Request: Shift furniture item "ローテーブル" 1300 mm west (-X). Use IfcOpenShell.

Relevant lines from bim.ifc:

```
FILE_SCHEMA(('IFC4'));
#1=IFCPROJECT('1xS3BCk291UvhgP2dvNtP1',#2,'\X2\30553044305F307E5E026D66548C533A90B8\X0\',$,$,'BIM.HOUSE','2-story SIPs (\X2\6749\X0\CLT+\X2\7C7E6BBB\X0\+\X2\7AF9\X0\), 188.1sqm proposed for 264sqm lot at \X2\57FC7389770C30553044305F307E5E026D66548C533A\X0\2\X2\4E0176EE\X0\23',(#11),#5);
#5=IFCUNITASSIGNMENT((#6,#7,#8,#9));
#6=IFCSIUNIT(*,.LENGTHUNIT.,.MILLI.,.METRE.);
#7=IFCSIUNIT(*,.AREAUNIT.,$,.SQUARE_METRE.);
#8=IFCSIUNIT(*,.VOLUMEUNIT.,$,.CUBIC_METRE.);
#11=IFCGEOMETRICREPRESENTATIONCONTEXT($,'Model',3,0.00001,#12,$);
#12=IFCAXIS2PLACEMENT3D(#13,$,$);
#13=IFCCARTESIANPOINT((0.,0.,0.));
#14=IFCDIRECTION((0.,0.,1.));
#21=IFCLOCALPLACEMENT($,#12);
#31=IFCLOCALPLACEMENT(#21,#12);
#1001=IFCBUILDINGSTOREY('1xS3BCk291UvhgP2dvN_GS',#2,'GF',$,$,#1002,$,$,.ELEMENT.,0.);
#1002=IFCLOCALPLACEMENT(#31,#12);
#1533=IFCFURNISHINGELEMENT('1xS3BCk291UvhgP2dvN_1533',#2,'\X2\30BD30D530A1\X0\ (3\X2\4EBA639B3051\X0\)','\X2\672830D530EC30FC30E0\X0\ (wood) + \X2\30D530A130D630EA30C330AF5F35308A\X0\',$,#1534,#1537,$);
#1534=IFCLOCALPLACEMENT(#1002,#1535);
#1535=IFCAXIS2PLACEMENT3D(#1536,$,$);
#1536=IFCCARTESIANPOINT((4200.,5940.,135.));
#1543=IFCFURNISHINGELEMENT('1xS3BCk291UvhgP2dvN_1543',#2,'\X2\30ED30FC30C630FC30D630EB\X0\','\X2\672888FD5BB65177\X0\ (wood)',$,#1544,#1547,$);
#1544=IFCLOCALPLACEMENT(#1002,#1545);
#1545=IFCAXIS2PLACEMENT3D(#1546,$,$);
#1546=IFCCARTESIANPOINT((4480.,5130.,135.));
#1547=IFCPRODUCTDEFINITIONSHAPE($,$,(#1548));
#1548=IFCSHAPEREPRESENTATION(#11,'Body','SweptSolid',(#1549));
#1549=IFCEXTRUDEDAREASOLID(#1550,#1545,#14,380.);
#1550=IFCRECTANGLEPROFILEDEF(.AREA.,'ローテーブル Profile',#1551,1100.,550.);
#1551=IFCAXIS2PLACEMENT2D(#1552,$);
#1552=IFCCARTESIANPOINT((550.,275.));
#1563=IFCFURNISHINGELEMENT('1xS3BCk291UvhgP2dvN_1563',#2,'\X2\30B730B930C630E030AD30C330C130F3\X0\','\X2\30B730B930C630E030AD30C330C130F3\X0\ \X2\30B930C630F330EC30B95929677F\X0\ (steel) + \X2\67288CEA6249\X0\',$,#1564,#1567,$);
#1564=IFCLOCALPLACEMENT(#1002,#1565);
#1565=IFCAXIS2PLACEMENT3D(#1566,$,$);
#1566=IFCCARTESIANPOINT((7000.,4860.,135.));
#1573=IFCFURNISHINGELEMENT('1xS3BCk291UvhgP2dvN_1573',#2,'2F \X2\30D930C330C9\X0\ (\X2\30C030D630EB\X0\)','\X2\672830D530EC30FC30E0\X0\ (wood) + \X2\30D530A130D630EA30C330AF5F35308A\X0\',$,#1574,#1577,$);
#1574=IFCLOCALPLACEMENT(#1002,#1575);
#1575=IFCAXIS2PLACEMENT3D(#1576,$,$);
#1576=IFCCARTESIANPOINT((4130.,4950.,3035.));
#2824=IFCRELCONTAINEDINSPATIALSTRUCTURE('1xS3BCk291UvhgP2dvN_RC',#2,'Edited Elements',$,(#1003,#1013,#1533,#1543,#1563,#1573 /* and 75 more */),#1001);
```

```python
import ifcopenshell
import ifcopenshell.api.geometry
import ifcopenshell.util.placement
import ifcopenshell.util.unit

model = ifcopenshell.open("bim.ifc")
unit_scale = ifcopenshell.util.unit.calculate_unit_scale(model)

item = model.by_guid("1xS3BCk291UvhgP2dvN_1543")
matrix = ifcopenshell.util.placement.get_local_placement(item.ObjectPlacement)
matrix[0, 3] -= 1.3 / unit_scale
ifcopenshell.api.geometry.edit_object_placement(model, product=item, matrix=matrix, is_si=False)

print(ifcopenshell.util.placement.get_local_placement(item.ObjectPlacement).round(3) + 0.0)

model.write("bim_updated.ifc")
```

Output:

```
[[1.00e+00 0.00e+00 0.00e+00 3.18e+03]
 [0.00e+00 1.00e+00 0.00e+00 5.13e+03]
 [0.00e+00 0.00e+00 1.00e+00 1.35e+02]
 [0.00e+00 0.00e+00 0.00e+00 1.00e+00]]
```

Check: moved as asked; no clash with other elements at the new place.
